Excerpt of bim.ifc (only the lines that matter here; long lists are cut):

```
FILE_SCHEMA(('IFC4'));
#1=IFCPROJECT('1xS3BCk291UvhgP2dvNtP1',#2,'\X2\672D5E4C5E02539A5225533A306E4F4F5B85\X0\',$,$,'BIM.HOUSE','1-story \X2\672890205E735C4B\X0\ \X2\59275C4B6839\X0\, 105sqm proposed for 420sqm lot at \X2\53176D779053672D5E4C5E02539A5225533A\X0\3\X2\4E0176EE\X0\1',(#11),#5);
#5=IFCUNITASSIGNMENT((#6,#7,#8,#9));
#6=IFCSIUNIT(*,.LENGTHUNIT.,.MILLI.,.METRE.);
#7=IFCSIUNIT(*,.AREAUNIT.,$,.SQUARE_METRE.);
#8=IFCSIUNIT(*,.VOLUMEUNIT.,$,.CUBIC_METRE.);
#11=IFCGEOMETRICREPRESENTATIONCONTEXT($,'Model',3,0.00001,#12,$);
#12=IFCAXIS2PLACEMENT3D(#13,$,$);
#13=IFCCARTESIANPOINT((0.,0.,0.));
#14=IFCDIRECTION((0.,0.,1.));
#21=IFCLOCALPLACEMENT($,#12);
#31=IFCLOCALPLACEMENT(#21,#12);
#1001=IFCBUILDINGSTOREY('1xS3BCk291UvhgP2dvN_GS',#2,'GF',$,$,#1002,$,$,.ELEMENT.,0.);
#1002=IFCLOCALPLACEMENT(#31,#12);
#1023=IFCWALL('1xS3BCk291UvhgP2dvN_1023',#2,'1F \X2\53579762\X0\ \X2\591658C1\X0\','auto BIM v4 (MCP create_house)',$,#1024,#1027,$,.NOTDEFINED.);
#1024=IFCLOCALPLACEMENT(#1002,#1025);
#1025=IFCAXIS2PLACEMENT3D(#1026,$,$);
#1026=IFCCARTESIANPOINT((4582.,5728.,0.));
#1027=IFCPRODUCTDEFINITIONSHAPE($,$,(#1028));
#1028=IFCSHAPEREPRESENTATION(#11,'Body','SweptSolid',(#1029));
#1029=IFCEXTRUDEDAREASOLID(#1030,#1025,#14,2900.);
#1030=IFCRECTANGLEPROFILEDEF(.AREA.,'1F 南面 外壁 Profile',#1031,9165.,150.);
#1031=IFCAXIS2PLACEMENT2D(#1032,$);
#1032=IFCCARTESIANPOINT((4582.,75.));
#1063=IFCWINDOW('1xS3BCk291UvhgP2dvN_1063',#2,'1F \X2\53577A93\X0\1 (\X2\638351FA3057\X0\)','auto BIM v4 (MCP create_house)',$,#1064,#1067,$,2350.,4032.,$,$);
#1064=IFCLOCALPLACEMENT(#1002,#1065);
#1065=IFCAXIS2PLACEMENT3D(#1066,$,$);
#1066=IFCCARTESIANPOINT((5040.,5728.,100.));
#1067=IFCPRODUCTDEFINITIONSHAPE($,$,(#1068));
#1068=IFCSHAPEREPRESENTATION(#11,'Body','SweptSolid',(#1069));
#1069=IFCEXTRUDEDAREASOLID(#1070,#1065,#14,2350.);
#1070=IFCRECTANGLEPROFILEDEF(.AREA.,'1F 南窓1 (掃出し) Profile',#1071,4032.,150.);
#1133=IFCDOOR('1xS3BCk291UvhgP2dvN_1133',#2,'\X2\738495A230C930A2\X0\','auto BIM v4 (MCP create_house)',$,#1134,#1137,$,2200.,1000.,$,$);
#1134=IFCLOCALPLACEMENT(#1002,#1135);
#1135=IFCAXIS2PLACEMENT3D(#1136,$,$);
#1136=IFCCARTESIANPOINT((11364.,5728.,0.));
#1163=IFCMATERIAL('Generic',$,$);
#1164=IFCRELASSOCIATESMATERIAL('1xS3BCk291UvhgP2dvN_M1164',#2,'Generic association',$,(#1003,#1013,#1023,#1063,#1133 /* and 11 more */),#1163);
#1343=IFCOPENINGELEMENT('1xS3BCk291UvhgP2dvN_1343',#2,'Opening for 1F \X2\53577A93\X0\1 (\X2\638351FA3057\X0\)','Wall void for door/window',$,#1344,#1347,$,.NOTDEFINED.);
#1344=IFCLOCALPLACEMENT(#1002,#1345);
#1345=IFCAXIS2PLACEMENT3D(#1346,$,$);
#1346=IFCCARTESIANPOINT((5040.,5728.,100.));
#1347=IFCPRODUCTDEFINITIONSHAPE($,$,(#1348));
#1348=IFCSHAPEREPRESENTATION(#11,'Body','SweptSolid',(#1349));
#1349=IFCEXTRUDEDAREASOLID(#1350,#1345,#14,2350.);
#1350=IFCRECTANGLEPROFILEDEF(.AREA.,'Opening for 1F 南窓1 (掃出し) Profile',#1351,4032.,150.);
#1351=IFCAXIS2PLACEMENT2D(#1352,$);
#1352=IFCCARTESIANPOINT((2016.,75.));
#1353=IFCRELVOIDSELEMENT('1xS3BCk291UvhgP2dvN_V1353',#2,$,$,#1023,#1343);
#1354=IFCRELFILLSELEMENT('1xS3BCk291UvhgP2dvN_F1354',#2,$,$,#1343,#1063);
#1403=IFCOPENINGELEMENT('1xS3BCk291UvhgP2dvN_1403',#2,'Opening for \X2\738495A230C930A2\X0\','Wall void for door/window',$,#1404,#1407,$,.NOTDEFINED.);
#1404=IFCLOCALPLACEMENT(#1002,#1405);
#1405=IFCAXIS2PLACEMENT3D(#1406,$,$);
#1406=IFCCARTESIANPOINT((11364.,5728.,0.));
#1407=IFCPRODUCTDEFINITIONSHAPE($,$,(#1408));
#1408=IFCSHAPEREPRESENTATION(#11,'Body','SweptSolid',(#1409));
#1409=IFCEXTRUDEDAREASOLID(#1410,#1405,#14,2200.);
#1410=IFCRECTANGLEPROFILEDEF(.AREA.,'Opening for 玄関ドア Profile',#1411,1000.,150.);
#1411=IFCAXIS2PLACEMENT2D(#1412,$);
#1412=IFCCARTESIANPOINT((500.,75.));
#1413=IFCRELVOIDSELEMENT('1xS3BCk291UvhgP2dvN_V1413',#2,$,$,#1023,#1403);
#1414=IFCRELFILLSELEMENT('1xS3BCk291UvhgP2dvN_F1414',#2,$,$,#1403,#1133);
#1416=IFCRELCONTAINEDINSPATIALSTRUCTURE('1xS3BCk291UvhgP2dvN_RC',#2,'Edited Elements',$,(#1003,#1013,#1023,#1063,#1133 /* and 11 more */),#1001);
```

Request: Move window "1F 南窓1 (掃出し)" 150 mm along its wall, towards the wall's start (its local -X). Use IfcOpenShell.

```python
import ifcopenshell
import ifcopenshell.api.geometry
import ifcopenshell.util.placement

model = ifcopenshell.open("bim.ifc")

window = model.by_guid("1xS3BCk291UvhgP2dvN_1063")
opening = window.FillsVoids[0].RelatingOpeningElement
wall = opening.VoidsElements[0].RelatingBuildingElement

wall_matrix = ifcopenshell.util.placement.get_local_placement(wall.ObjectPlacement)
shift = wall_matrix[:3, 0] * -150.0
before = ifcopenshell.util.placement.get_local_placement(window.ObjectPlacement)[:3, 3].copy()

# The window is not placed relative to its opening, so move both.
for product in (opening, window):
    matrix = ifcopenshell.util.placement.get_local_placement(product.ObjectPlacement)
    matrix[:3, 3] += shift
    ifcopenshell.api.geometry.edit_object_placement(model, product=product, matrix=matrix, is_si=False)

after = ifcopenshell.util.placement.get_local_placement(window.ObjectPlacement)[:3, 3]
print("window moved by", (after - before).round(3) + 0.0)

model.write("bim_rev.ifc")
```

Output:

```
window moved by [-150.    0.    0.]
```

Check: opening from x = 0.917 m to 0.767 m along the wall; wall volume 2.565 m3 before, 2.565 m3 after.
